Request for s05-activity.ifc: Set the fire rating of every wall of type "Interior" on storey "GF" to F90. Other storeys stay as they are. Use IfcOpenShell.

First a look at what the model holds.

```python
import ifcopenshell
import ifcopenshell.util.element

model = ifcopenshell.open("s05-activity.ifc")
print(model.schema)
storey = next(s for s in model.by_type("IfcBuildingStorey") if s.Name == "GF")
walls = [e for e in ifcopenshell.util.element.get_decomposition(storey) if e.is_a("IfcWall")]
seen = {}
for e in walls:
    element_type = ifcopenshell.util.element.get_type(e)
    key = (element_type.Name if element_type != e and element_type else None, ifcopenshell.util.element.get_pset(e, "Pset_WallCommon", "FireRating"))
    seen[key] = seen.get(key, 0) + 1
for (name, value), count in sorted(seen.items(), key=str):
    print(count, "x", name, "|", value)
```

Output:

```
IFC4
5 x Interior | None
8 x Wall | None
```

```python
import ifcopenshell
import ifcopenshell.api.pset
import ifcopenshell.util.element

model = ifcopenshell.open("s05-activity.ifc")

storey = next(s for s in model.by_type("IfcBuildingStorey") if s.Name == "GF")
walls = [e for e in ifcopenshell.util.element.get_decomposition(storey) if e.is_a("IfcWall")]

count = 0
for e in walls:
    element_type = ifcopenshell.util.element.get_type(e)
    if element_type in (None, e) or element_type.Name != "Interior":
        continue
    # add_pset returns the element's existing set when there is one.
    pset = ifcopenshell.api.pset.add_pset(model, product=e, name="Pset_WallCommon")
    ifcopenshell.api.pset.edit_pset(model, pset=pset, properties={"FireRating": "F90"})
    count += 1

print(count, "walls updated")

model.write("s05-activity-out.ifc")
```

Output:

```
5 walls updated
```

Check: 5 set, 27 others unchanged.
